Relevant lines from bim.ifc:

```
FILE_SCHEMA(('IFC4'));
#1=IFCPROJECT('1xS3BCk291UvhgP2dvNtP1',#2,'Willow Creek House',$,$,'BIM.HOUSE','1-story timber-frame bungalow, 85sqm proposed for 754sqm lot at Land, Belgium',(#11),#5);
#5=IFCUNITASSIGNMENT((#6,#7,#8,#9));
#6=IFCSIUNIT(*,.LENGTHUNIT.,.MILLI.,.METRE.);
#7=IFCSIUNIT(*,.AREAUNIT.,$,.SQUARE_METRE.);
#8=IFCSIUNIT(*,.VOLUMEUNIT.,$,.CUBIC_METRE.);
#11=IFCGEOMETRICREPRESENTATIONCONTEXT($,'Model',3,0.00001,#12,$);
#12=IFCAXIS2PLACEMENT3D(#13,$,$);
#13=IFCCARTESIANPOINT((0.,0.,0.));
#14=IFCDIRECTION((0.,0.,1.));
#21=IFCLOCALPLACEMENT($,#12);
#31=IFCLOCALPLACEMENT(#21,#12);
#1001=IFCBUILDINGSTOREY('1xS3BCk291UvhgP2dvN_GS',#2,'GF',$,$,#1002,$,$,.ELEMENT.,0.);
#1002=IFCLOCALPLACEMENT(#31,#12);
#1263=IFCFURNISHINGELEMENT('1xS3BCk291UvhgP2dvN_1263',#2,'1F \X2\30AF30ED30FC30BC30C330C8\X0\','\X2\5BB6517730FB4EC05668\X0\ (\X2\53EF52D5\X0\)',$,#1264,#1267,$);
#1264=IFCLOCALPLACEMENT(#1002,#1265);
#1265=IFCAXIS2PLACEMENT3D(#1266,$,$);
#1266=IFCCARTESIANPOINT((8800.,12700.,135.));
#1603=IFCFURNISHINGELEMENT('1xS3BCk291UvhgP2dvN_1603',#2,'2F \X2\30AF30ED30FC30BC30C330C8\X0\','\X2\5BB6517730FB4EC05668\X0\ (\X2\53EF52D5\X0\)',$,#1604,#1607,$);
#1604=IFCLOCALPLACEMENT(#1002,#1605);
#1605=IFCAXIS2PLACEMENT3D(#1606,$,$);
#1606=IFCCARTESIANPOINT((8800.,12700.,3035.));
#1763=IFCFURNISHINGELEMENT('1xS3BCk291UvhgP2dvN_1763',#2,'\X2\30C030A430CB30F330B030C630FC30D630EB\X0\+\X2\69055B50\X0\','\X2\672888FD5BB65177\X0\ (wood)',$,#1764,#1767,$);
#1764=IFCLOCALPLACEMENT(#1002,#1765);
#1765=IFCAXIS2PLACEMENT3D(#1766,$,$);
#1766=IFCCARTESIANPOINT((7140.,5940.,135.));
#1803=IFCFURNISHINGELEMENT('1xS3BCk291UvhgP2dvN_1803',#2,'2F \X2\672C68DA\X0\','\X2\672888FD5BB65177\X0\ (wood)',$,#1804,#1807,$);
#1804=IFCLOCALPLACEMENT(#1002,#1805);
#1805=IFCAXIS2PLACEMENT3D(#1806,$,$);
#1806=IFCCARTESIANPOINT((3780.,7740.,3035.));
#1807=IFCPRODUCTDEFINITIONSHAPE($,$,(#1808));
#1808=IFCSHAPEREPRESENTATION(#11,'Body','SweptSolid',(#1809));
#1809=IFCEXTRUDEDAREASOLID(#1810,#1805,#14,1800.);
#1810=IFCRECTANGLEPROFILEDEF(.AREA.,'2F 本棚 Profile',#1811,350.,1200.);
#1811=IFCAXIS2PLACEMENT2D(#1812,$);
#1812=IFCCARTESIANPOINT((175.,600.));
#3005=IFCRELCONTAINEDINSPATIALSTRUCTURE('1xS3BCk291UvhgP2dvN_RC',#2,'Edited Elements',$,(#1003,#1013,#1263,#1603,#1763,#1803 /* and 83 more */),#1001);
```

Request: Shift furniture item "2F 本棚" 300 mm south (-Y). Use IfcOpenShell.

```python
import ifcopenshell
import ifcopenshell.api.geometry
import ifcopenshell.util.placement

model = ifcopenshell.open("bim.ifc")

item = model.by_id(1803)
matrix = ifcopenshell.util.placement.get_local_placement(item.ObjectPlacement)
matrix[1, 3] -= 300.0
ifcopenshell.api.geometry.edit_object_placement(model, product=item, matrix=matrix, is_si=False)

print(ifcopenshell.util.placement.get_local_placement(item.ObjectPlacement).round(3) + 0.0)

model.write("bim_updated.ifc")
```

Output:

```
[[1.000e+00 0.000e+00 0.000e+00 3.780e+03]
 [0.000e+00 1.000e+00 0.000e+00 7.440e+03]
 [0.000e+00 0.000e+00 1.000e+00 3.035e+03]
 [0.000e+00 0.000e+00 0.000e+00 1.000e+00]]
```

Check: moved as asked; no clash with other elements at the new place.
